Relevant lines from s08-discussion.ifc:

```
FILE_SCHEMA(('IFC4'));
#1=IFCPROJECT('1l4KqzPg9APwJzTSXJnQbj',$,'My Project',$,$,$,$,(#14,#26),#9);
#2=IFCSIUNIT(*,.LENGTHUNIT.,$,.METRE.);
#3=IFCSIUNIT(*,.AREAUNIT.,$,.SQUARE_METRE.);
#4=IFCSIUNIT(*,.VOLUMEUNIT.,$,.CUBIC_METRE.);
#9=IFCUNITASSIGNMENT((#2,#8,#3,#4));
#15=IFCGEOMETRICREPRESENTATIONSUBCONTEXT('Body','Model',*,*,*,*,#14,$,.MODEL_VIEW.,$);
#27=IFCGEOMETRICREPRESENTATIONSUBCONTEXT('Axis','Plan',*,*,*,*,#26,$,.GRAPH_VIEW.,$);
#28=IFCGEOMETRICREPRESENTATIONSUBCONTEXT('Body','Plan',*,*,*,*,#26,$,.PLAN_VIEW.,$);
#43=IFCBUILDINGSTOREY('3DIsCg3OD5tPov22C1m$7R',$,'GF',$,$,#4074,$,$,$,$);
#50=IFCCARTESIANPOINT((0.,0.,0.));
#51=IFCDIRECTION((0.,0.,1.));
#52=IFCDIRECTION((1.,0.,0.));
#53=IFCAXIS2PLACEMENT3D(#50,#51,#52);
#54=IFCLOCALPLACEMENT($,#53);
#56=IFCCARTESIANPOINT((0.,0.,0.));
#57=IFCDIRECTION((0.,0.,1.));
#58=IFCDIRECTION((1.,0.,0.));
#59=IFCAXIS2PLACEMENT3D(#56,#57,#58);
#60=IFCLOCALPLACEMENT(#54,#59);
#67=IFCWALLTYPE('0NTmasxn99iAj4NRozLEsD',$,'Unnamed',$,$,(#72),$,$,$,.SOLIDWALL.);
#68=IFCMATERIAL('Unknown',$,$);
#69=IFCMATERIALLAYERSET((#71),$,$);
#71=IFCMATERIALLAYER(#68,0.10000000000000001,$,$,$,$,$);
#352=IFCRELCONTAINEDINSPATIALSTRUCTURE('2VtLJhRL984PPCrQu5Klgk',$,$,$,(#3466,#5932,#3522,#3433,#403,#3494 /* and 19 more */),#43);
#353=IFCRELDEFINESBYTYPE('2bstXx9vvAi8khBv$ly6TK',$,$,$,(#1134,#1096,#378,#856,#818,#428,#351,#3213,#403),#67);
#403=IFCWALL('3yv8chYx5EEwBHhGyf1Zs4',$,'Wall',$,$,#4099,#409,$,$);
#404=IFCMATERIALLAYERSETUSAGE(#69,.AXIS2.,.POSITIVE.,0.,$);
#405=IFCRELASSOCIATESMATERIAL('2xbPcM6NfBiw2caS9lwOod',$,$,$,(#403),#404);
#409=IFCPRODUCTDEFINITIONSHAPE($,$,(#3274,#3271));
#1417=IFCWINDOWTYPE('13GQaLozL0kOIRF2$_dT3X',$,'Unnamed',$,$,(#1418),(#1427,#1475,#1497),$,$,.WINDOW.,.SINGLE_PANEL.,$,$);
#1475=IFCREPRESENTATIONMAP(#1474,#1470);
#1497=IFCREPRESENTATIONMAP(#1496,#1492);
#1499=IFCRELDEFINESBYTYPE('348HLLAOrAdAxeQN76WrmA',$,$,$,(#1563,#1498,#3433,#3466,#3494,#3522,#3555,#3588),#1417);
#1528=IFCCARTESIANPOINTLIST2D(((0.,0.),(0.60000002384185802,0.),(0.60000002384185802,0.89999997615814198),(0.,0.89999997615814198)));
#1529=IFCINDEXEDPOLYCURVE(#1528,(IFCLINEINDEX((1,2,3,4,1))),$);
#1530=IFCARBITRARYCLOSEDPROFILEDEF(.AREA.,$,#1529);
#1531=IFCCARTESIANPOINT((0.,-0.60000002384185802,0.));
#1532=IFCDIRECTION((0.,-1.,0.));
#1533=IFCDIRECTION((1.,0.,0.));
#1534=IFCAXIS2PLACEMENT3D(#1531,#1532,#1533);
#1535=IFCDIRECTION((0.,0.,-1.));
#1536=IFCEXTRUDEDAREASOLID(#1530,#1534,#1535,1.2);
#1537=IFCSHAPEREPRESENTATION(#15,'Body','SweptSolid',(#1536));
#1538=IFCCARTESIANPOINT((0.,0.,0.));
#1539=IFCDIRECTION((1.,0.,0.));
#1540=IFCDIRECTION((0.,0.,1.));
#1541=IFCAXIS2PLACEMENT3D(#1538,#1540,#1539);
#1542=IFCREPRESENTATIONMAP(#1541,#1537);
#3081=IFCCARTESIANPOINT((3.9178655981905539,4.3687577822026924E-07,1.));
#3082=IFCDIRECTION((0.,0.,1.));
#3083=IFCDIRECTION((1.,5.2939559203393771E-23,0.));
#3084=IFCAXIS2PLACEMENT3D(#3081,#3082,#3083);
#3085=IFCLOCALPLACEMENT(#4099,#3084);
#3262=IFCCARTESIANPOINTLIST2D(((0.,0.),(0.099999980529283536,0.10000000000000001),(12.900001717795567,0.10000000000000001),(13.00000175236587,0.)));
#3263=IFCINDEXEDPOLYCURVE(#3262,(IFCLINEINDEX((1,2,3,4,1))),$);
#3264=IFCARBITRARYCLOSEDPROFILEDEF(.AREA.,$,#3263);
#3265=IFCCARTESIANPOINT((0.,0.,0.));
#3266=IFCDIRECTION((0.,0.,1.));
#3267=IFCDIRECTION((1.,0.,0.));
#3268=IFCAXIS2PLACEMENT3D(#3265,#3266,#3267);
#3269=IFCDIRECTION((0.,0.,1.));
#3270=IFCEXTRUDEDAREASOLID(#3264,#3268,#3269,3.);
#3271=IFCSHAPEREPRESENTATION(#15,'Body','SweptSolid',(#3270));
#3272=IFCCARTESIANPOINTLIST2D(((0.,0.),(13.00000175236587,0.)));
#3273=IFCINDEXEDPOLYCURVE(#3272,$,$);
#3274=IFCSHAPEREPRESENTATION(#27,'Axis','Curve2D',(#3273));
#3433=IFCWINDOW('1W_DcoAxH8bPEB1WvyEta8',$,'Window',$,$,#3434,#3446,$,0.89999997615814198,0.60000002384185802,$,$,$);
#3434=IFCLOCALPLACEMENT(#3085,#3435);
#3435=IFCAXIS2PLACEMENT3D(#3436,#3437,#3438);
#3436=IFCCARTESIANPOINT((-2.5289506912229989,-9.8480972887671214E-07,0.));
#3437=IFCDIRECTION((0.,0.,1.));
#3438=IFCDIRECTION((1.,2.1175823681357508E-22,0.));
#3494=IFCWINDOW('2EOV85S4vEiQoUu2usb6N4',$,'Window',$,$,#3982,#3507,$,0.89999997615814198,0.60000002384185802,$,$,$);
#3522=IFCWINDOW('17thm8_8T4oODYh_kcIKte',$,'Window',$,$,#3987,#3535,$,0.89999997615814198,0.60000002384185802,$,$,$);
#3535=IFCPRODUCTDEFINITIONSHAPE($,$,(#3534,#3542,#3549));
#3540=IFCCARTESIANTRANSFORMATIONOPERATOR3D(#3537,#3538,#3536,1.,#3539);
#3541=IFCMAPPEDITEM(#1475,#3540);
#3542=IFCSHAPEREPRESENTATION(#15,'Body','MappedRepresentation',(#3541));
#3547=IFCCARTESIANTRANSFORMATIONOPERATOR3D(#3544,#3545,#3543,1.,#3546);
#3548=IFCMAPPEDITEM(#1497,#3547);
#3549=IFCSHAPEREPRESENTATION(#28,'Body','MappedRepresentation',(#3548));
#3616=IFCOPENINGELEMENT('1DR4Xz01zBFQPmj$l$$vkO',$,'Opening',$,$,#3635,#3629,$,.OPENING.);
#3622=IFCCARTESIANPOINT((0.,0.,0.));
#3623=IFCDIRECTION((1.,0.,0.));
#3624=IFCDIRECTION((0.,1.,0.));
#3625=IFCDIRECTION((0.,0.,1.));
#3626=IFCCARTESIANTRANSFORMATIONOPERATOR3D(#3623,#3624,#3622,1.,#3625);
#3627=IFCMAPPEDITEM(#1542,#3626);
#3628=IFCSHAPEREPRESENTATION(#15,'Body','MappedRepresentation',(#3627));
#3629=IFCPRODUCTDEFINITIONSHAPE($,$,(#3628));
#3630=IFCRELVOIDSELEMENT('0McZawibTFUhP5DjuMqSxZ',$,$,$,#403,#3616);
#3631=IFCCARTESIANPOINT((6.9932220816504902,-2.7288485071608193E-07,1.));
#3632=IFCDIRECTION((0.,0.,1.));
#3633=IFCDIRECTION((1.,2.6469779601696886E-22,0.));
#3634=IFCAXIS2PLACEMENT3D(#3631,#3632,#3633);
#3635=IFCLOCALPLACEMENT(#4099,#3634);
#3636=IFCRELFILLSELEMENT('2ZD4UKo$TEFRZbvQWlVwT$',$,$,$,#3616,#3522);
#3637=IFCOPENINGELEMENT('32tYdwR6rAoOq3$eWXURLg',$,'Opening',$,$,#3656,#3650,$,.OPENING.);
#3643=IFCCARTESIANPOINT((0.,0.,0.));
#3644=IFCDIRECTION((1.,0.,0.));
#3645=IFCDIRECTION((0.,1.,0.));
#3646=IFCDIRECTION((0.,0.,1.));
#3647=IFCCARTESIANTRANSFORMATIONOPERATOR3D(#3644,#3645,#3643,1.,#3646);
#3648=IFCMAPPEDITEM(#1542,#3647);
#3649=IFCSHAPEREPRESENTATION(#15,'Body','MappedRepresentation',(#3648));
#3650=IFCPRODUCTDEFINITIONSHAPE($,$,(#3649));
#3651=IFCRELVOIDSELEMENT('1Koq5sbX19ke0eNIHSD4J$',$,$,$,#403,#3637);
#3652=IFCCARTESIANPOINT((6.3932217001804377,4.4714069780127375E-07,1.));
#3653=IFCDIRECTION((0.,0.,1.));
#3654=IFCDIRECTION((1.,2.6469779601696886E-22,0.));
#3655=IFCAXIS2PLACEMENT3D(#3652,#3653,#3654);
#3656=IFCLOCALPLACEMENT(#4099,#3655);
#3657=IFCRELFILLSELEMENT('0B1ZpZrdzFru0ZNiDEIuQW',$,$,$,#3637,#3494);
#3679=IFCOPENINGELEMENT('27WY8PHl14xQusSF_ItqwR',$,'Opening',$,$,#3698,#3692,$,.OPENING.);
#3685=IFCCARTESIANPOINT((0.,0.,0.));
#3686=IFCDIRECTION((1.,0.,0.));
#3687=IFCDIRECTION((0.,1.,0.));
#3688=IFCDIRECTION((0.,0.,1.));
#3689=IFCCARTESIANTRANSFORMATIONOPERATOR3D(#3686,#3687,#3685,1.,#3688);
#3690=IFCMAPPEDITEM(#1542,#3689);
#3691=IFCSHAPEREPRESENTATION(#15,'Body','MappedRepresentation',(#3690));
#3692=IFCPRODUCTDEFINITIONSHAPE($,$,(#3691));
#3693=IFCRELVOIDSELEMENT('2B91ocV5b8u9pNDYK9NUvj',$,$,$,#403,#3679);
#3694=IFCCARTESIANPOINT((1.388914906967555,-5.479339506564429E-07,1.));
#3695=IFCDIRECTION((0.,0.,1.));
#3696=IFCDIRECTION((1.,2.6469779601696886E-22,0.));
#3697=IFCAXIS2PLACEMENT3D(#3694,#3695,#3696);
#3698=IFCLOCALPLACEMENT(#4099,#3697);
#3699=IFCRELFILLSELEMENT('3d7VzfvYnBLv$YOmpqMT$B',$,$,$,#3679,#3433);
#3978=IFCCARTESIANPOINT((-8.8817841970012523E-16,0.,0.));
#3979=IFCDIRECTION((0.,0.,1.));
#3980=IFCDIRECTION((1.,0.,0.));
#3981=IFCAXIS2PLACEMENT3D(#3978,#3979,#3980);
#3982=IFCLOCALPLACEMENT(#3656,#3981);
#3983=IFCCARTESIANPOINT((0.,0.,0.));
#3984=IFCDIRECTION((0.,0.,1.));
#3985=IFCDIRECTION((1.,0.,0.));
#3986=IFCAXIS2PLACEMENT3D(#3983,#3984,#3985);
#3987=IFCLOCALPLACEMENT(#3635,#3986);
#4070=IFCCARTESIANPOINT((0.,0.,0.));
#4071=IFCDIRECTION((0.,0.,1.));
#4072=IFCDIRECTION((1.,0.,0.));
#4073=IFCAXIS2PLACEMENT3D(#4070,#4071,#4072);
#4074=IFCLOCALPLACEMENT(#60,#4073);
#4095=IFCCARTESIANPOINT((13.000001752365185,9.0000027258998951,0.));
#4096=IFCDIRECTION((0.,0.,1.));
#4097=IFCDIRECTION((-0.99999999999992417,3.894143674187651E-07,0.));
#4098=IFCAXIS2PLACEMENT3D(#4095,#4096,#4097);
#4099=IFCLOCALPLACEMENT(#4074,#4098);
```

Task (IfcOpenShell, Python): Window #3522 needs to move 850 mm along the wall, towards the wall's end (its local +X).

```python
import ifcopenshell
import ifcopenshell.api.geometry
import ifcopenshell.util.placement
import ifcopenshell.util.unit

model = ifcopenshell.open("s08-discussion.ifc")
unit_scale = ifcopenshell.util.unit.calculate_unit_scale(model)

window = model.by_guid("17thm8_8T4oODYh_kcIKte")
opening = window.FillsVoids[0].RelatingOpeningElement
wall = opening.VoidsElements[0].RelatingBuildingElement

wall_matrix = ifcopenshell.util.placement.get_local_placement(wall.ObjectPlacement)
shift = wall_matrix[:3, 0] * 0.85 / unit_scale
before = ifcopenshell.util.placement.get_local_placement(window.ObjectPlacement)[:3, 3].copy()

# The window is placed relative to its opening, so it follows when the opening moves.
matrix = ifcopenshell.util.placement.get_local_placement(opening.ObjectPlacement)
matrix[:3, 3] += shift
ifcopenshell.api.geometry.edit_object_placement(
    model, product=opening, matrix=matrix, is_si=False, should_transform_children=True
)

after = ifcopenshell.util.placement.get_local_placement(window.ObjectPlacement)[:3, 3]
print("window moved by", (after - before).round(3) + 0.0)

model.write("s08-discussion_v2.ifc")
```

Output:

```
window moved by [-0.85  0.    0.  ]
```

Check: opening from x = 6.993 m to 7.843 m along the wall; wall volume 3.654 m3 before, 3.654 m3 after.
